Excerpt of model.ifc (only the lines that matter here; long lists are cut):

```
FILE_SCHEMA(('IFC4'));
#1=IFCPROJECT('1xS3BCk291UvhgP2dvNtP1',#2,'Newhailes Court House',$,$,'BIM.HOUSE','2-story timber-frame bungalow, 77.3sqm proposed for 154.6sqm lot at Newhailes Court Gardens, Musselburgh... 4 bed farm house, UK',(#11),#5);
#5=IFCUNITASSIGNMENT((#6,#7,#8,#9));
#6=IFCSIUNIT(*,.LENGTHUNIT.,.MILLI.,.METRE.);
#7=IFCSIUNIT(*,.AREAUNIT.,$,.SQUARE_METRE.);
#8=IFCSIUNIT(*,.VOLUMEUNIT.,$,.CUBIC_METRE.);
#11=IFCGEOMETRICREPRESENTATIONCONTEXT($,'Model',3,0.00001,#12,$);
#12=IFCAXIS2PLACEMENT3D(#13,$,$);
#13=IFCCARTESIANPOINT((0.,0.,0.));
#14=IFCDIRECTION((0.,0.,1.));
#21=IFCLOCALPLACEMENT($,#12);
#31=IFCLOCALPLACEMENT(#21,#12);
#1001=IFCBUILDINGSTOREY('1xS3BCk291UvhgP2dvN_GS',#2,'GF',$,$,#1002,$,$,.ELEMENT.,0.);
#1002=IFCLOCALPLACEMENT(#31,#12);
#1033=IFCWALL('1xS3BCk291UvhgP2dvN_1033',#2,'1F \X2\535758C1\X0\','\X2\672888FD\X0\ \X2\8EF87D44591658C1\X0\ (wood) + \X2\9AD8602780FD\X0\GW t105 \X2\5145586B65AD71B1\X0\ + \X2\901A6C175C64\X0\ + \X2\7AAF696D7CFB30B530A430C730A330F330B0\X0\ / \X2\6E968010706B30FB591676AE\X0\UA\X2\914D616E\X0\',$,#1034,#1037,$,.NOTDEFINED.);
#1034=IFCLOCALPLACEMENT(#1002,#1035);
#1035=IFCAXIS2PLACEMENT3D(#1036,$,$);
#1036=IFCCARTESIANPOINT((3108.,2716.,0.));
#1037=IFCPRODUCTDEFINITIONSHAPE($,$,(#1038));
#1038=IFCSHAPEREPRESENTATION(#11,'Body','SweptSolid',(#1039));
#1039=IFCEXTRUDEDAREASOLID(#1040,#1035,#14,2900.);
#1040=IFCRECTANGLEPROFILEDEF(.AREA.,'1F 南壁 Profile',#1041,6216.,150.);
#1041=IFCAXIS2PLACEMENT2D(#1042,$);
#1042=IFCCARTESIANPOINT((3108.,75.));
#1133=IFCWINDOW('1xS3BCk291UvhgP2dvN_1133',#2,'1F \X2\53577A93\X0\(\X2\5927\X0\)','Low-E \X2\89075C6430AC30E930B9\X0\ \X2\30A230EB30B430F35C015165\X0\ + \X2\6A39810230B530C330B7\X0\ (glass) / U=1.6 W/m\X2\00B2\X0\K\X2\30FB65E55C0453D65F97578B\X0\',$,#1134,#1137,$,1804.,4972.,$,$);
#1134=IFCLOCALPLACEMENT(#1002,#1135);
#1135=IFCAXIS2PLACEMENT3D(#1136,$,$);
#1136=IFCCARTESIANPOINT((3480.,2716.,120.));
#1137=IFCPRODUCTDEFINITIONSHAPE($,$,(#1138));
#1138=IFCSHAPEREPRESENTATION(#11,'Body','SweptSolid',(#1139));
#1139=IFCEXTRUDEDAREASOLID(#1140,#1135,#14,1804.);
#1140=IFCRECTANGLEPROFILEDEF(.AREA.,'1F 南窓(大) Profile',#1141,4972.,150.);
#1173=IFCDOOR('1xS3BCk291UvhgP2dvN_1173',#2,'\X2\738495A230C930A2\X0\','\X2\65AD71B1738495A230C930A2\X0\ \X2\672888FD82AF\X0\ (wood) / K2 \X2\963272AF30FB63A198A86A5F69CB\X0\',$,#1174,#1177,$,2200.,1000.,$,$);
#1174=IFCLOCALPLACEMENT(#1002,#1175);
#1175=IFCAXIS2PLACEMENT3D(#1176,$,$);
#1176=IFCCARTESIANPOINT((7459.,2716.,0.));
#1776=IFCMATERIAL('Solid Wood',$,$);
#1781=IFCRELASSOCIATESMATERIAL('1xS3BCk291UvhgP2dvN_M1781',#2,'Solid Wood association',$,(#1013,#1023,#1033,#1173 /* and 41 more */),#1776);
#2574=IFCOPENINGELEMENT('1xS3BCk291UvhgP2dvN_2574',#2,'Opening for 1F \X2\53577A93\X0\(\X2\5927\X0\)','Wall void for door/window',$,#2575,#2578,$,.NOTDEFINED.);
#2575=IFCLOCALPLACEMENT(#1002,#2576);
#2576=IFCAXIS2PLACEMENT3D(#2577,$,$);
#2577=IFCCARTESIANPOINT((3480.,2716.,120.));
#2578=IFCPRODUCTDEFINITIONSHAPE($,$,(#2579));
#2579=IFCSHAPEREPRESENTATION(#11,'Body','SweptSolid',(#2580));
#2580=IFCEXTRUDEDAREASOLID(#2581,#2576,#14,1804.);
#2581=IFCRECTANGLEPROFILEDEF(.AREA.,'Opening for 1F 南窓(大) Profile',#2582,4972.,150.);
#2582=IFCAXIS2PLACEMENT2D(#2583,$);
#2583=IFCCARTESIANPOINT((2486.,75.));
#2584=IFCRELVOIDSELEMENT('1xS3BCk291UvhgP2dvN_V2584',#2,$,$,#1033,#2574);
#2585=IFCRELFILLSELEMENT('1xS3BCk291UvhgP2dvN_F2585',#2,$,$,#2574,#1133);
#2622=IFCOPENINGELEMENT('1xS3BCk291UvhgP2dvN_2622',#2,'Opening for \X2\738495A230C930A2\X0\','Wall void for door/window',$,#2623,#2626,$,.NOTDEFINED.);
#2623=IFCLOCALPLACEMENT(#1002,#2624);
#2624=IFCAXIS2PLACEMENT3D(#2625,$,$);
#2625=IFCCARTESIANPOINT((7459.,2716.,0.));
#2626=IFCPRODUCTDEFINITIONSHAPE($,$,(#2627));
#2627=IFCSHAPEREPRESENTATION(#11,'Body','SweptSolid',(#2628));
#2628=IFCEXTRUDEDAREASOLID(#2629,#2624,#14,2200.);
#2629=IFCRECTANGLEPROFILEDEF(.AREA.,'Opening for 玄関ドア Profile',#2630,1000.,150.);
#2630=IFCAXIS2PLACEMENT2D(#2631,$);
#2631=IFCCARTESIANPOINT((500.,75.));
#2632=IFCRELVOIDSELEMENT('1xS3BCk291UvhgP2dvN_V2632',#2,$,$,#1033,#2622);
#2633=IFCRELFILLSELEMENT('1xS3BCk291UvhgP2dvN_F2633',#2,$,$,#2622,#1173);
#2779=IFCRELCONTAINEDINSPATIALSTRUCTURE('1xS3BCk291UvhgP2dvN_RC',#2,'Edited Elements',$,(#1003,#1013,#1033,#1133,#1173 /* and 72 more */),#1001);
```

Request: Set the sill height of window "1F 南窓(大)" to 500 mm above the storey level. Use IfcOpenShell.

```python
import numpy as np
import ifcopenshell
import ifcopenshell.api.geometry
import ifcopenshell.geom
import ifcopenshell.util.element
import ifcopenshell.util.placement
import ifcopenshell.util.shape
import ifcopenshell.util.unit

model = ifcopenshell.open("model.ifc")
unit_scale = ifcopenshell.util.unit.calculate_unit_scale(model)

window = model.by_id(1133)
opening = window.FillsVoids[0].RelatingOpeningElement
storey = ifcopenshell.util.element.get_container(window, ifc_class="IfcBuildingStorey")
level = ifcopenshell.util.placement.get_local_placement(storey.ObjectPlacement)[2, 3]

# The opening's origin need not be at the sill, so measure its lowest point.
shape = ifcopenshell.geom.create_shape(ifcopenshell.geom.settings(), opening)
bottom = ifcopenshell.util.shape.get_shape_bottom_elevation(shape, shape.geometry) / unit_scale
dz = level + 0.5 / unit_scale - bottom

shift = np.array([0.0, 0.0, dz])
# The window is not placed relative to its opening, so move both.
for product in (opening, window):
    matrix = ifcopenshell.util.placement.get_local_placement(product.ObjectPlacement)
    matrix[:3, 3] += shift
    ifcopenshell.api.geometry.edit_object_placement(model, product=product, matrix=matrix, is_si=False)

print(f"moved by {dz * unit_scale:+.3f} m")

model.write("model_edited.ifc")
```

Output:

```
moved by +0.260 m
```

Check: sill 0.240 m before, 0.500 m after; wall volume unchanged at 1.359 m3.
